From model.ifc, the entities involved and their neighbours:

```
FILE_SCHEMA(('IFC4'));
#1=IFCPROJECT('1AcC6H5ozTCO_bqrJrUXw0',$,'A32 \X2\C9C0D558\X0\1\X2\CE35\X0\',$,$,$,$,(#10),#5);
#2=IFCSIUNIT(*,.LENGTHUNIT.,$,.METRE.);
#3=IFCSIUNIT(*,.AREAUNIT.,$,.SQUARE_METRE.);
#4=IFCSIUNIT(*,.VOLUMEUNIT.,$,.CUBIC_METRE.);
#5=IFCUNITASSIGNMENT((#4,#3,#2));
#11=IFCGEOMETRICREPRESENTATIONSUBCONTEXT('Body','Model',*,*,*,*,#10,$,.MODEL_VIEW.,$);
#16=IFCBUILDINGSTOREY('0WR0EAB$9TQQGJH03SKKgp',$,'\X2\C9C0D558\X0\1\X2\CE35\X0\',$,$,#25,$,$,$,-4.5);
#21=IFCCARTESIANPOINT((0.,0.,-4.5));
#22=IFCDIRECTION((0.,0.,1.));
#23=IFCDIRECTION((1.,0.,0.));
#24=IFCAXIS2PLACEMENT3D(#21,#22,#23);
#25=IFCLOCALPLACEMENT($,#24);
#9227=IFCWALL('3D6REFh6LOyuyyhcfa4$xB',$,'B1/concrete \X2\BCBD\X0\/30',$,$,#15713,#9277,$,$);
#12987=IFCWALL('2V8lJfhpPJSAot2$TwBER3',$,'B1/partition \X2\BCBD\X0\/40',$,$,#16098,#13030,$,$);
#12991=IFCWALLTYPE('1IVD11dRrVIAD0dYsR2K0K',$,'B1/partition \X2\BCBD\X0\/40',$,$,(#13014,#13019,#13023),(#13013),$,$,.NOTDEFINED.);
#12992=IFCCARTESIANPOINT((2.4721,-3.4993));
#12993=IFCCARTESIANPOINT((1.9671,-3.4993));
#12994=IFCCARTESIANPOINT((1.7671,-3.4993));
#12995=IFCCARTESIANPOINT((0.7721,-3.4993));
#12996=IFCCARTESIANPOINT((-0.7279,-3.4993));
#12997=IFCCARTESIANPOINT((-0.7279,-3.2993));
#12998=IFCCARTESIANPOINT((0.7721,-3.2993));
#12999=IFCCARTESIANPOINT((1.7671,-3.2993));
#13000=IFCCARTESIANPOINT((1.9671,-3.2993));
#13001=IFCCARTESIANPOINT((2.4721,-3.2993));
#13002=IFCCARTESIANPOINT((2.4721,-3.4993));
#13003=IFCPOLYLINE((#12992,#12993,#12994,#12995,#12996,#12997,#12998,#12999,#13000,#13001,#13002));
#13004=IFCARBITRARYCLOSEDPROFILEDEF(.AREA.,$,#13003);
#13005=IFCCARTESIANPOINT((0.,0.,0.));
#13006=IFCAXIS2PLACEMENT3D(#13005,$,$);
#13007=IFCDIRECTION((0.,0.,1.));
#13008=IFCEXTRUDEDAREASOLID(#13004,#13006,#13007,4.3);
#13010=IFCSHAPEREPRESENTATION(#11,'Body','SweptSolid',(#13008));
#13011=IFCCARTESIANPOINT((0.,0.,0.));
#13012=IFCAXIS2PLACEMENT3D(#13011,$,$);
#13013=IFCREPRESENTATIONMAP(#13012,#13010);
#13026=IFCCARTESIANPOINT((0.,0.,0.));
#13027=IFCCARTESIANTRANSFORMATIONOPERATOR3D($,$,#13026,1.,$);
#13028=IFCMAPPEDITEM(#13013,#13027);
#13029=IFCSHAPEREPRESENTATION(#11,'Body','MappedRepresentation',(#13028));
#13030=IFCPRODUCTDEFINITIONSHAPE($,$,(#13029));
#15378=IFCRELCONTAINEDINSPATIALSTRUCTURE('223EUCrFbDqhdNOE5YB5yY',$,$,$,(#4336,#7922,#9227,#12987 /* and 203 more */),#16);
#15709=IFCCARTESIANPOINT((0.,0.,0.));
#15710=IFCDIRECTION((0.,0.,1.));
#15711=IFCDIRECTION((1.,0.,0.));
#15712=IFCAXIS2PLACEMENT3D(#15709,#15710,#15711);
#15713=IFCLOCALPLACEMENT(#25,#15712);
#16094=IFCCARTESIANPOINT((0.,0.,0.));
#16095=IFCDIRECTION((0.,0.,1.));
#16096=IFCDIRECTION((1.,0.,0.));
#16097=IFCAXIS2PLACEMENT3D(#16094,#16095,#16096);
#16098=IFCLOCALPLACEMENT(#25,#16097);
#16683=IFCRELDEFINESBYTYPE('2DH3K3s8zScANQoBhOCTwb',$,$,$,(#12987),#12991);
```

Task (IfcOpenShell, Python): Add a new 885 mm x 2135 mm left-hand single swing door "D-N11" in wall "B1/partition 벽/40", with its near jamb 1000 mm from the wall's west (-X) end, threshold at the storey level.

```python
import numpy as np
import ifcopenshell
import ifcopenshell.api.feature
import ifcopenshell.api.geometry
import ifcopenshell.api.root
import ifcopenshell.api.spatial
import ifcopenshell.geom
import ifcopenshell.util.element
import ifcopenshell.util.placement
import ifcopenshell.util.representation
import ifcopenshell.util.shape
import ifcopenshell.util.unit

model = ifcopenshell.open("model.ifc")
unit_scale = ifcopenshell.util.unit.calculate_unit_scale(model)
settings = ifcopenshell.geom.settings()


def volume(element):
    """Net volume in cubic metres, openings subtracted."""
    shape = ifcopenshell.geom.create_shape(settings, element)
    return ifcopenshell.util.shape.get_volume(shape.geometry)


wall = model.by_guid("2V8lJfhpPJSAot2$TwBER3")
storey = ifcopenshell.util.element.get_container(wall, ifc_class="IfcBuildingStorey")
context = ifcopenshell.util.representation.get_context(model, "Model", "Body", "MODEL_VIEW")
before = volume(wall)

width, height, from_end, sill = 0.885, 2.135, 1, 0.0  # metres

# The wall runs along its own X axis, and the end named is its -X end.
wall_shape = ifcopenshell.geom.create_shape(settings, wall)
x, y, z = ifcopenshell.util.shape.get_vertices(wall_shape.geometry).T
start = x.min() + from_end
face, thickness = float(y.min()), float(y.max() - y.min())
wall_matrix = ifcopenshell.util.placement.get_local_placement(wall.ObjectPlacement)
level = ifcopenshell.util.placement.get_local_placement(storey.ObjectPlacement)[2, 3]


def in_wall(x, y):
    """Placement at x, y metres in the wall's axes, at sill height."""
    matrix = wall_matrix.copy()
    matrix[:, 3] = wall_matrix @ np.array([x / unit_scale, y / unit_scale, 0.0, 1.0])
    matrix[2, 3] = level + sill / unit_scale
    return matrix


# Opening: a box that overshoots both wall faces by 50 mm.
opening = ifcopenshell.api.root.create_entity(model, ifc_class="IfcOpeningElement", predefined_type="OPENING")
box = ifcopenshell.api.geometry.add_wall_representation(
    model, context=context, length=width, height=height, thickness=thickness + 0.1
)
ifcopenshell.api.geometry.assign_representation(model, product=opening, representation=box)
ifcopenshell.api.geometry.edit_object_placement(model, product=opening, matrix=in_wall(start, face - 0.05), is_si=False)
ifcopenshell.api.feature.add_feature(model, feature=opening, element=wall)

door = ifcopenshell.api.root.create_entity(model, ifc_class="IfcDoor", name="D-N11", predefined_type="DOOR")
door.OverallWidth, door.OverallHeight = width / unit_scale, height / unit_scale
door.OperationType = "SINGLE_SWING_LEFT"
body = ifcopenshell.api.geometry.add_door_representation(
    model,
    context=context,
    overall_width=door.OverallWidth,
    overall_height=door.OverallHeight,
    operation_type="SINGLE_SWING_LEFT",
    lining_properties={"LiningDepth": thickness / unit_scale, "ThresholdDepth": thickness / unit_scale},
)
ifcopenshell.api.geometry.assign_representation(model, product=door, representation=body)
ifcopenshell.api.spatial.assign_container(model, products=[door], relating_structure=storey)
ifcopenshell.api.feature.add_filling(model, opening=opening, element=door)

# The lining spans the wall, so the door starts at the wall face.
ifcopenshell.api.geometry.edit_object_placement(model, product=door, matrix=in_wall(start, face), is_si=False)

after = volume(wall)

print(f"wall volume {before:.3f} -> {after:.3f} m3")

model.write("model_rev.ifc")
```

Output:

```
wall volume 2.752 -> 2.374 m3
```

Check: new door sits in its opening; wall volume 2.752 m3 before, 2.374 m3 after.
